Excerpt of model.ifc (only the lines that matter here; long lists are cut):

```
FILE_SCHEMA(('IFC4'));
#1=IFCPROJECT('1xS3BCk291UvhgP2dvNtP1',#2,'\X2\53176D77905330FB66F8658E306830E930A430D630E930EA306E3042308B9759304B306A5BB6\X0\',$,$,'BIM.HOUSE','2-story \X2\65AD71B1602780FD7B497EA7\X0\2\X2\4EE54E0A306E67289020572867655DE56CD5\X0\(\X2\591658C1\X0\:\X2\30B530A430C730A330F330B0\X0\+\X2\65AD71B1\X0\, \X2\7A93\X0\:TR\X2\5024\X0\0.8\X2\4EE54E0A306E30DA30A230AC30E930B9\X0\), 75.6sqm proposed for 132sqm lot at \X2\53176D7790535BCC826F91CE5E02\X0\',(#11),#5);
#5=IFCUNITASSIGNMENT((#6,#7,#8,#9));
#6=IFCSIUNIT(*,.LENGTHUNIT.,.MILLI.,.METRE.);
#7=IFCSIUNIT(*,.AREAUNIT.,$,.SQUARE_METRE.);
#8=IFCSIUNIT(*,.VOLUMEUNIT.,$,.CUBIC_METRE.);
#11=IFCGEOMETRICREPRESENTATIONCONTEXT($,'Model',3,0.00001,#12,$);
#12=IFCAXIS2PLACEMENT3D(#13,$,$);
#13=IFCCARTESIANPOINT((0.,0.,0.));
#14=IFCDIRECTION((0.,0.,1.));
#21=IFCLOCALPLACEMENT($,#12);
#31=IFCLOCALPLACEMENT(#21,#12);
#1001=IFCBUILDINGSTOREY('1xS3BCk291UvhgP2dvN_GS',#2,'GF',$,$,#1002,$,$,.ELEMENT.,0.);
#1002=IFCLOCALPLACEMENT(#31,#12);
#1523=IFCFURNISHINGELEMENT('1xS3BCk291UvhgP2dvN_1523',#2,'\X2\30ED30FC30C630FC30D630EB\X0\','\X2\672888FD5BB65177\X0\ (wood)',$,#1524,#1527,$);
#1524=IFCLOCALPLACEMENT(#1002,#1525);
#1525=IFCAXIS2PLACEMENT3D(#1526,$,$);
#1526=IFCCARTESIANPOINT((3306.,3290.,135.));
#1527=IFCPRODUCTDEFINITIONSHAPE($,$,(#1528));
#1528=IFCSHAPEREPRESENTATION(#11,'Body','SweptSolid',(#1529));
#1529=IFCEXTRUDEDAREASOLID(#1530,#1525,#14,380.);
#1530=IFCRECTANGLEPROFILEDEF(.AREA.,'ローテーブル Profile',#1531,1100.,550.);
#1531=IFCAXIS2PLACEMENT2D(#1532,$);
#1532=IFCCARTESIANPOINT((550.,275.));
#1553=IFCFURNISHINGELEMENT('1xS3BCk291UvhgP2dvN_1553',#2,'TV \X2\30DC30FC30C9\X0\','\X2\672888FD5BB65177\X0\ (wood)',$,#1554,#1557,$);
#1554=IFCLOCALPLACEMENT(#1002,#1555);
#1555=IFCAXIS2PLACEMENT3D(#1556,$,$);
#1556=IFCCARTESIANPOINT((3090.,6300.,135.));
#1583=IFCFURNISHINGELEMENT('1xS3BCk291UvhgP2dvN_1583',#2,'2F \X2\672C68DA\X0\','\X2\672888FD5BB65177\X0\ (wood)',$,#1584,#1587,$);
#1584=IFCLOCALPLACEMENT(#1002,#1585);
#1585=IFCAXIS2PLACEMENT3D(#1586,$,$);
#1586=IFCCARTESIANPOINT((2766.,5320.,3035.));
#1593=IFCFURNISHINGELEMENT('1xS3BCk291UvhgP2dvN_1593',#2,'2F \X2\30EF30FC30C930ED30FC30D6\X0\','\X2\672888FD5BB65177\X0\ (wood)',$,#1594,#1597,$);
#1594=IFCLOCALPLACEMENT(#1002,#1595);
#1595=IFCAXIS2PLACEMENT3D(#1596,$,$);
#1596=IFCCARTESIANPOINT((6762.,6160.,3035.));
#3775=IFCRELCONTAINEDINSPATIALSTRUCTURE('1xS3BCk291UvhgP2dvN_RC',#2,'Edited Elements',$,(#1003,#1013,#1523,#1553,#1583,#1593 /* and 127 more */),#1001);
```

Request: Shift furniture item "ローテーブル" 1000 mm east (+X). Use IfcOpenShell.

```python
import ifcopenshell
import ifcopenshell.api.geometry
import ifcopenshell.util.placement
import ifcopenshell.util.unit

model = ifcopenshell.open("model.ifc")
unit_scale = ifcopenshell.util.unit.calculate_unit_scale(model)

item = model.by_guid("1xS3BCk291UvhgP2dvN_1523")
matrix = ifcopenshell.util.placement.get_local_placement(item.ObjectPlacement)
matrix[0, 3] += 1 / unit_scale
ifcopenshell.api.geometry.edit_object_placement(model, product=item, matrix=matrix, is_si=False)

print(ifcopenshell.util.placement.get_local_placement(item.ObjectPlacement).round(3) + 0.0)

model.write("model_rev.ifc")
```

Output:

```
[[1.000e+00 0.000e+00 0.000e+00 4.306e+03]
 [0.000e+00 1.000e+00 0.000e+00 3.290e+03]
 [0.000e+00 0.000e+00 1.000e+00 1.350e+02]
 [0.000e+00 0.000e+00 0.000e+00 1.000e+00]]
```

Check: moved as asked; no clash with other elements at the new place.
